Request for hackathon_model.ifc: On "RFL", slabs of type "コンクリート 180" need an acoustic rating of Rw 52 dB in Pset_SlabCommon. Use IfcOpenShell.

First a look at what the model holds.

```python
import ifcopenshell
import ifcopenshell.util.element

model = ifcopenshell.open("hackathon_model.ifc")
print(model.schema)
storey = next(s for s in model.by_type("IfcBuildingStorey") if s.Name == "RFL")
slabs = [e for e in ifcopenshell.util.element.get_decomposition(storey) if e.is_a("IfcSlab")]
seen = {}
for e in slabs:
    element_type = ifcopenshell.util.element.get_type(e)
    key = (element_type.Name if element_type != e and element_type else None, ifcopenshell.util.element.get_pset(e, "Pset_SlabCommon", "AcousticRating"))
    seen[key] = seen.get(key, 0) + 1
for (name, value), count in sorted(seen.items(), key=str):
    print(count, "x", name, "|", value)
```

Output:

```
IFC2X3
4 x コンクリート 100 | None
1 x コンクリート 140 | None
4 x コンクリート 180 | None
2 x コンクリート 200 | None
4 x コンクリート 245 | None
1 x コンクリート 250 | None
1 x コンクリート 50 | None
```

```python
import ifcopenshell
import ifcopenshell.api.pset
import ifcopenshell.util.element

model = ifcopenshell.open("hackathon_model.ifc")

storey = next(s for s in model.by_type("IfcBuildingStorey") if s.Name == "RFL")
slabs = [e for e in ifcopenshell.util.element.get_decomposition(storey) if e.is_a("IfcSlab")]

count = 0
for e in slabs:
    element_type = ifcopenshell.util.element.get_type(e)
    if element_type in (None, e) or element_type.Name != "コンクリート 180":
        continue
    # add_pset returns the element's existing set when there is one.
    pset = ifcopenshell.api.pset.add_pset(model, product=e, name="Pset_SlabCommon")
    ifcopenshell.api.pset.edit_pset(model, pset=pset, properties={"AcousticRating": "Rw 52 dB"})
    count += 1

print(count, "slabs updated")

model.write("hackathon_model_updated.ifc")
```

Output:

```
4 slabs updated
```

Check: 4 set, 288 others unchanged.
